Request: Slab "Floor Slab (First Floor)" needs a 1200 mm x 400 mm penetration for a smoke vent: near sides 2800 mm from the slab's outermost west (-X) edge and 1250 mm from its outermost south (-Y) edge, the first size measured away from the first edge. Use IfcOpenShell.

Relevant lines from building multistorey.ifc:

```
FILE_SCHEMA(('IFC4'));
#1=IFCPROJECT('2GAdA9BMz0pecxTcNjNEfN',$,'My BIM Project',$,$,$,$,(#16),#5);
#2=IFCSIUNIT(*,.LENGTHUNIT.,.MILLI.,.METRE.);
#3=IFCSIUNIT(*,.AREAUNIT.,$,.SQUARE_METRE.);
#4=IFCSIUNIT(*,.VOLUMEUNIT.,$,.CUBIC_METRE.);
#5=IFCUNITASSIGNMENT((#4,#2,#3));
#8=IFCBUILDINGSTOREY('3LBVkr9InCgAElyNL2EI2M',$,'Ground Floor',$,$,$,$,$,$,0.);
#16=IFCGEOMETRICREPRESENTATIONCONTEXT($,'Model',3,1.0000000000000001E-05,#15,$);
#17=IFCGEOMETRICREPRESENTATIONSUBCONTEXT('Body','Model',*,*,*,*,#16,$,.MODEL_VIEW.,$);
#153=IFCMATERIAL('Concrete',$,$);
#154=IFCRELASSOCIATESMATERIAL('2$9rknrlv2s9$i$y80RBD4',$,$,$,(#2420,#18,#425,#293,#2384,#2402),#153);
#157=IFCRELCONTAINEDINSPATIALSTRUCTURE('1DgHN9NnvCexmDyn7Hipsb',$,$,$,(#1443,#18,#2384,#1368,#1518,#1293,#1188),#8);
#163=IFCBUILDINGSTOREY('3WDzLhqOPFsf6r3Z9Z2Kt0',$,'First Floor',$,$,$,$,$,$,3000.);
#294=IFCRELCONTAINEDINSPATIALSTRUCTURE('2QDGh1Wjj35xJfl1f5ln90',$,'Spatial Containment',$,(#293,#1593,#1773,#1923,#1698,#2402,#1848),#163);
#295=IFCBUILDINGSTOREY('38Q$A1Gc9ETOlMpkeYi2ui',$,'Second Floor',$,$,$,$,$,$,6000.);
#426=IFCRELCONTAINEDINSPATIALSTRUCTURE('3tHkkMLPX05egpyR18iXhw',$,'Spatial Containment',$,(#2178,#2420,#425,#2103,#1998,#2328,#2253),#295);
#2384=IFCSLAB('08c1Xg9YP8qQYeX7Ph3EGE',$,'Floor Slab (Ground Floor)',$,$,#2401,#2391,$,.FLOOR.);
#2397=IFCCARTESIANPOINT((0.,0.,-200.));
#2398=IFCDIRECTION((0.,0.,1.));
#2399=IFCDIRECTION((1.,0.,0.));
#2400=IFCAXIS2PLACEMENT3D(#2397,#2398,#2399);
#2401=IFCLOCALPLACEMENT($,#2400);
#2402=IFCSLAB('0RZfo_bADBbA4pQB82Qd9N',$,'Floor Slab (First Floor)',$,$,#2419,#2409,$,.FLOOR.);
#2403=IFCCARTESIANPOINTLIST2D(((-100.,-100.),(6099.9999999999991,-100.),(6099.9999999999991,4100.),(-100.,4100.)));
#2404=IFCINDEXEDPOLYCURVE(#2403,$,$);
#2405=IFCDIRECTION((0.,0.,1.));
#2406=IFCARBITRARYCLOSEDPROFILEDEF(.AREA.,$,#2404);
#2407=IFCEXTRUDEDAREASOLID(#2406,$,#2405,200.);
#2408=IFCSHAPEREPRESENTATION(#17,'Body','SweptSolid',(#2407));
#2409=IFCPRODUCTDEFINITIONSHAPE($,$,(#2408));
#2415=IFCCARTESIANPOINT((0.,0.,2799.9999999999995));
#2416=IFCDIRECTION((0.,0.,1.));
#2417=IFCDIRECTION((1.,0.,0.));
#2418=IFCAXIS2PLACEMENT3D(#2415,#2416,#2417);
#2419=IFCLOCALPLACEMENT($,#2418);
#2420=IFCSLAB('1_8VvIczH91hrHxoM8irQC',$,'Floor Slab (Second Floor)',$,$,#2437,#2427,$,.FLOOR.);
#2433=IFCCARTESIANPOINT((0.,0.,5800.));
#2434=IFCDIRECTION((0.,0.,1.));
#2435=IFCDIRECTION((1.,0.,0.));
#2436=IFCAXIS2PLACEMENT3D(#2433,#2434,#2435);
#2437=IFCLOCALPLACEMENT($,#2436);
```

```python
import numpy as np
import ifcopenshell
import ifcopenshell.api.feature
import ifcopenshell.api.geometry
import ifcopenshell.api.root
import ifcopenshell.geom
import ifcopenshell.util.placement
import ifcopenshell.util.representation
import ifcopenshell.util.shape
import ifcopenshell.util.unit

model = ifcopenshell.open("building multistorey.ifc")
unit_scale = ifcopenshell.util.unit.calculate_unit_scale(model)
settings = ifcopenshell.geom.settings()


def volume(element):
    """Net volume in cubic metres, openings subtracted."""
    shape = ifcopenshell.geom.create_shape(settings, element)
    return ifcopenshell.util.shape.get_volume(shape.geometry)


slab = model.by_id(2402)
before = volume(slab)

# Extent in the slab's own axes, in metres. The edges named are its -X and -Y sides.
slab_shape = ifcopenshell.geom.create_shape(settings, slab)
vertices = ifcopenshell.util.shape.get_vertices(slab_shape.geometry)
x_min, y_min, bottom = vertices.min(axis=0)
top = vertices[:, 2].max()

opening = ifcopenshell.api.root.create_entity(model, ifc_class="IfcOpeningElement", name="Smoke vent opening", predefined_type="OPENING")
context = ifcopenshell.util.representation.get_context(model, "Model", "Body", "MODEL_VIEW")
width, depth = 1.2, 0.4
outline = [(0.0, 0.0), (width, 0.0), (width, depth), (0.0, depth), (0.0, 0.0)]
# Overshoot both faces by 50 mm so the cut is clean.
shape = ifcopenshell.api.geometry.add_slab_representation(
    model, context=context, depth=top - bottom + 0.1, polyline=outline
)
ifcopenshell.api.geometry.assign_representation(model, product=opening, representation=shape)

matrix = ifcopenshell.util.placement.get_local_placement(slab.ObjectPlacement)
matrix[:, 3] = matrix @ np.append(np.array([x_min + 2.8, y_min + 1.25, bottom - 0.05]) / unit_scale, 1.0)
ifcopenshell.api.geometry.edit_object_placement(model, product=opening, matrix=matrix, is_si=False)
ifcopenshell.api.feature.add_feature(model, feature=opening, element=slab)

after = volume(slab)

print(f"slab volume {before:.3f} -> {after:.3f} m3")

model.write("building multistorey_v2.ifc")
```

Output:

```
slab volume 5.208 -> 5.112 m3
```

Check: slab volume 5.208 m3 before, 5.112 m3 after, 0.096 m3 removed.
